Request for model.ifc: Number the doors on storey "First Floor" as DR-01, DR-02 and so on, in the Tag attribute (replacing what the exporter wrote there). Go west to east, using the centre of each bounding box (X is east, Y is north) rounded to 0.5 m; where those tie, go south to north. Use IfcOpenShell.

First a look at what the model holds.

```python
import ifcopenshell
import ifcopenshell.util.element
import ifcopenshell.util.placement

model = ifcopenshell.open("model.ifc")
print(model.schema)
storey = next(s for s in model.by_type("IfcBuildingStorey") if s.Name == "First Floor")
doors = [e for e in ifcopenshell.util.element.get_decomposition(storey) if e.is_a("IfcDoor")]
for e in sorted(doors, key=lambda e: e.id()):
    origin = ifcopenshell.util.placement.get_local_placement(e.ObjectPlacement)[:3, 3]
    print(e.id(), e.Tag, e.Name, origin.round(2) + 0.0, sep=" | ")
```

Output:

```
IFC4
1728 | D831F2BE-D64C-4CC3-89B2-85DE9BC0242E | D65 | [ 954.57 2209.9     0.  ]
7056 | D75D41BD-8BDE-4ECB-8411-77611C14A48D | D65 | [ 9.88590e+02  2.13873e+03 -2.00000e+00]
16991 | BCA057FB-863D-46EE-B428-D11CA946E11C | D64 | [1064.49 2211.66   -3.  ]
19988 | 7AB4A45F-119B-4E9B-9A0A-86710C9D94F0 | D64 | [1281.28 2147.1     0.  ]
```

```python
import ifcopenshell
import ifcopenshell.geom
import ifcopenshell.util.element
import ifcopenshell.util.shape

model = ifcopenshell.open("model.ifc")
settings = ifcopenshell.geom.settings()
settings.set("use-world-coords", True)


def centre(element):
    shape = ifcopenshell.geom.create_shape(settings, element)
    return ifcopenshell.util.shape.get_bbox_centroid(shape.geometry)


storey = next(s for s in model.by_type("IfcBuildingStorey") if s.Name == "First Floor")
doors = [e for e in ifcopenshell.util.element.get_decomposition(storey) if e.is_a("IfcDoor")]

# Insertion points can sit at a corner or the storey origin, so sort by the geometry (in metres).
centres = {e: centre(e) for e in doors}
doors.sort(key=lambda e: (round(centres[e][0] / 0.5), centres[e][1]))

for i, e in enumerate(doors, start=1):
    number = f"DR-{i:02d}"
    e.Tag = number
    print(e.id(), number)

model.write("model_edited.ifc")
```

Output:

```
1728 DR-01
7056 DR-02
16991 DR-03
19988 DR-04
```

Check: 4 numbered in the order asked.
